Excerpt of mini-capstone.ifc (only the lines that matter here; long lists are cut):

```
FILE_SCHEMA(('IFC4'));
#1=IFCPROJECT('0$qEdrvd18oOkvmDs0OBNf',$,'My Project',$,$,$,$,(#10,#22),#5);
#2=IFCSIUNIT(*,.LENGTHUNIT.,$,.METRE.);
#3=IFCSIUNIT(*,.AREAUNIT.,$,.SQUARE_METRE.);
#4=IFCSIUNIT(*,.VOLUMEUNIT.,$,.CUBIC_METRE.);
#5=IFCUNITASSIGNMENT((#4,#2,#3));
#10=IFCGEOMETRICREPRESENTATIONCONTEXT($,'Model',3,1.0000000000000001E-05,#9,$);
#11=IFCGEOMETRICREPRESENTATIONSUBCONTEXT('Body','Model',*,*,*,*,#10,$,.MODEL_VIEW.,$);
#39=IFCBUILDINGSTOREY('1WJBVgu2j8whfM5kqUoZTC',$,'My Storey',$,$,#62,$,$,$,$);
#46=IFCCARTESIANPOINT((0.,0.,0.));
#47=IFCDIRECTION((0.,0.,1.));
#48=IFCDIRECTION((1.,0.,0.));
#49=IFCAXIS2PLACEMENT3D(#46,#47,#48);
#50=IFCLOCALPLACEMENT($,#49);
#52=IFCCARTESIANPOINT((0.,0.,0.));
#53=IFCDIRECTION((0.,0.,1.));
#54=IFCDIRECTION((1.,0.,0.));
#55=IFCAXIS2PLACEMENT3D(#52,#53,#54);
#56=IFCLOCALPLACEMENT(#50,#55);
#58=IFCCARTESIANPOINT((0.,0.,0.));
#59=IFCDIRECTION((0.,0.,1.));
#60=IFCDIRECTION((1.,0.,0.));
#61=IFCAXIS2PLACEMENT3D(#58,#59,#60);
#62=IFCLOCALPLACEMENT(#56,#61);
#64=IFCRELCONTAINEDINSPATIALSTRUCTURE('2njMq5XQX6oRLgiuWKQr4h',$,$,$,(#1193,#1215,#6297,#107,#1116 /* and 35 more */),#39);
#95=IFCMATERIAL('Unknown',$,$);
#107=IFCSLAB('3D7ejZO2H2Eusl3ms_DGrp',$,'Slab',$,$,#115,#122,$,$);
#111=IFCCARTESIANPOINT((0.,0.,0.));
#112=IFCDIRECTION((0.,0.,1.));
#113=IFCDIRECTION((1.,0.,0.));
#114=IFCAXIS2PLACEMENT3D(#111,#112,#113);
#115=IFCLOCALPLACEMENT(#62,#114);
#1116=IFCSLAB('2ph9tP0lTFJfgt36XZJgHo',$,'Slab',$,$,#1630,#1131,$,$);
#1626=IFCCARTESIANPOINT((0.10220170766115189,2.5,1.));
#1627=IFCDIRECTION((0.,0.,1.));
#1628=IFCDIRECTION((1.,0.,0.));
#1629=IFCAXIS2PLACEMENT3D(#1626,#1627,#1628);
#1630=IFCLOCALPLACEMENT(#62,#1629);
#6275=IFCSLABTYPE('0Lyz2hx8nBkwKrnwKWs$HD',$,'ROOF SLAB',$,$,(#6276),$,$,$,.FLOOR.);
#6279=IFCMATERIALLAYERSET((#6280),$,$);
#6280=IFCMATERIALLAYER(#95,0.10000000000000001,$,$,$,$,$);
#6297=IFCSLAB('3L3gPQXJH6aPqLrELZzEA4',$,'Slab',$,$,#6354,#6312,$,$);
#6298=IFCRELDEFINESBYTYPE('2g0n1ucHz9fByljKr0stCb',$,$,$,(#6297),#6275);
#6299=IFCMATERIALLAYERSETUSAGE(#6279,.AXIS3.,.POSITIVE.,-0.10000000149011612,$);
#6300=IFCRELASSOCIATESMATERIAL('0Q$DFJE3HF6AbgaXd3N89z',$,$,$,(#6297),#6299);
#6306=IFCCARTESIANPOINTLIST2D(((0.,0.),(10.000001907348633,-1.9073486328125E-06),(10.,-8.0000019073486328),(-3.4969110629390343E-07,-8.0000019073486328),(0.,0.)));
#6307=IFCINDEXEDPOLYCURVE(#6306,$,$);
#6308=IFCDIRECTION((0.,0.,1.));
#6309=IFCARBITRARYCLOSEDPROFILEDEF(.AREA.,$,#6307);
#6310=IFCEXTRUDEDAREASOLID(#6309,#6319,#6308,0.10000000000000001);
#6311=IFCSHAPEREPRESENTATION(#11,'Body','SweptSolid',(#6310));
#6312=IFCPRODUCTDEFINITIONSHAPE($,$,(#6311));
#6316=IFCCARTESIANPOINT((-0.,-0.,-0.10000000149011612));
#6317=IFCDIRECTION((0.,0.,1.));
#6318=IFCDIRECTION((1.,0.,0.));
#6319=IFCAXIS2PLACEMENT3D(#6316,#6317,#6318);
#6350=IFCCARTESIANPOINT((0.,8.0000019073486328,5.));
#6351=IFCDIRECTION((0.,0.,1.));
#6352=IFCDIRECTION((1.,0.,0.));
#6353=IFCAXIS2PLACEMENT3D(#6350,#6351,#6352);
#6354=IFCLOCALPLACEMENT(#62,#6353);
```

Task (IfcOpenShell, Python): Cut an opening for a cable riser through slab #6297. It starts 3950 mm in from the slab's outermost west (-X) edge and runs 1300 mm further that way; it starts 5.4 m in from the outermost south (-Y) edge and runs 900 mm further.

```python
import numpy as np
import ifcopenshell
import ifcopenshell.api.feature
import ifcopenshell.api.geometry
import ifcopenshell.api.root
import ifcopenshell.geom
import ifcopenshell.util.placement
import ifcopenshell.util.representation
import ifcopenshell.util.shape
import ifcopenshell.util.unit

model = ifcopenshell.open("mini-capstone.ifc")
unit_scale = ifcopenshell.util.unit.calculate_unit_scale(model)
settings = ifcopenshell.geom.settings()


def volume(element):
    """Net volume in cubic metres, openings subtracted."""
    shape = ifcopenshell.geom.create_shape(settings, element)
    return ifcopenshell.util.shape.get_volume(shape.geometry)


slab = model.by_guid("3L3gPQXJH6aPqLrELZzEA4")
before = volume(slab)

# Extent in the slab's own axes, in metres. The edges named are its -X and -Y sides.
slab_shape = ifcopenshell.geom.create_shape(settings, slab)
vertices = ifcopenshell.util.shape.get_vertices(slab_shape.geometry)
x_min, y_min, bottom = vertices.min(axis=0)
top = vertices[:, 2].max()

opening = ifcopenshell.api.root.create_entity(model, ifc_class="IfcOpeningElement", name="Cable riser opening", predefined_type="OPENING")
context = ifcopenshell.util.representation.get_context(model, "Model", "Body", "MODEL_VIEW")
width, depth = 1.3, 0.9
outline = [(0.0, 0.0), (width, 0.0), (width, depth), (0.0, depth), (0.0, 0.0)]
# Overshoot both faces by 50 mm so the cut is clean.
shape = ifcopenshell.api.geometry.add_slab_representation(
    model, context=context, depth=top - bottom + 0.1, polyline=outline
)
ifcopenshell.api.geometry.assign_representation(model, product=opening, representation=shape)

matrix = ifcopenshell.util.placement.get_local_placement(slab.ObjectPlacement)
matrix[:, 3] = matrix @ np.append(np.array([x_min + 3.95, y_min + 5.4, bottom - 0.05]) / unit_scale, 1.0)
ifcopenshell.api.geometry.edit_object_placement(model, product=opening, matrix=matrix, is_si=False)
ifcopenshell.api.feature.add_feature(model, feature=opening, element=slab)

after = volume(slab)

print(f"slab volume {before:.3f} -> {after:.3f} m3")

model.write("mini-capstone_v2.ifc")
```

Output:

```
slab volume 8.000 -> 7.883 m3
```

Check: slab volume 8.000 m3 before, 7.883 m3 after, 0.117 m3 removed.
